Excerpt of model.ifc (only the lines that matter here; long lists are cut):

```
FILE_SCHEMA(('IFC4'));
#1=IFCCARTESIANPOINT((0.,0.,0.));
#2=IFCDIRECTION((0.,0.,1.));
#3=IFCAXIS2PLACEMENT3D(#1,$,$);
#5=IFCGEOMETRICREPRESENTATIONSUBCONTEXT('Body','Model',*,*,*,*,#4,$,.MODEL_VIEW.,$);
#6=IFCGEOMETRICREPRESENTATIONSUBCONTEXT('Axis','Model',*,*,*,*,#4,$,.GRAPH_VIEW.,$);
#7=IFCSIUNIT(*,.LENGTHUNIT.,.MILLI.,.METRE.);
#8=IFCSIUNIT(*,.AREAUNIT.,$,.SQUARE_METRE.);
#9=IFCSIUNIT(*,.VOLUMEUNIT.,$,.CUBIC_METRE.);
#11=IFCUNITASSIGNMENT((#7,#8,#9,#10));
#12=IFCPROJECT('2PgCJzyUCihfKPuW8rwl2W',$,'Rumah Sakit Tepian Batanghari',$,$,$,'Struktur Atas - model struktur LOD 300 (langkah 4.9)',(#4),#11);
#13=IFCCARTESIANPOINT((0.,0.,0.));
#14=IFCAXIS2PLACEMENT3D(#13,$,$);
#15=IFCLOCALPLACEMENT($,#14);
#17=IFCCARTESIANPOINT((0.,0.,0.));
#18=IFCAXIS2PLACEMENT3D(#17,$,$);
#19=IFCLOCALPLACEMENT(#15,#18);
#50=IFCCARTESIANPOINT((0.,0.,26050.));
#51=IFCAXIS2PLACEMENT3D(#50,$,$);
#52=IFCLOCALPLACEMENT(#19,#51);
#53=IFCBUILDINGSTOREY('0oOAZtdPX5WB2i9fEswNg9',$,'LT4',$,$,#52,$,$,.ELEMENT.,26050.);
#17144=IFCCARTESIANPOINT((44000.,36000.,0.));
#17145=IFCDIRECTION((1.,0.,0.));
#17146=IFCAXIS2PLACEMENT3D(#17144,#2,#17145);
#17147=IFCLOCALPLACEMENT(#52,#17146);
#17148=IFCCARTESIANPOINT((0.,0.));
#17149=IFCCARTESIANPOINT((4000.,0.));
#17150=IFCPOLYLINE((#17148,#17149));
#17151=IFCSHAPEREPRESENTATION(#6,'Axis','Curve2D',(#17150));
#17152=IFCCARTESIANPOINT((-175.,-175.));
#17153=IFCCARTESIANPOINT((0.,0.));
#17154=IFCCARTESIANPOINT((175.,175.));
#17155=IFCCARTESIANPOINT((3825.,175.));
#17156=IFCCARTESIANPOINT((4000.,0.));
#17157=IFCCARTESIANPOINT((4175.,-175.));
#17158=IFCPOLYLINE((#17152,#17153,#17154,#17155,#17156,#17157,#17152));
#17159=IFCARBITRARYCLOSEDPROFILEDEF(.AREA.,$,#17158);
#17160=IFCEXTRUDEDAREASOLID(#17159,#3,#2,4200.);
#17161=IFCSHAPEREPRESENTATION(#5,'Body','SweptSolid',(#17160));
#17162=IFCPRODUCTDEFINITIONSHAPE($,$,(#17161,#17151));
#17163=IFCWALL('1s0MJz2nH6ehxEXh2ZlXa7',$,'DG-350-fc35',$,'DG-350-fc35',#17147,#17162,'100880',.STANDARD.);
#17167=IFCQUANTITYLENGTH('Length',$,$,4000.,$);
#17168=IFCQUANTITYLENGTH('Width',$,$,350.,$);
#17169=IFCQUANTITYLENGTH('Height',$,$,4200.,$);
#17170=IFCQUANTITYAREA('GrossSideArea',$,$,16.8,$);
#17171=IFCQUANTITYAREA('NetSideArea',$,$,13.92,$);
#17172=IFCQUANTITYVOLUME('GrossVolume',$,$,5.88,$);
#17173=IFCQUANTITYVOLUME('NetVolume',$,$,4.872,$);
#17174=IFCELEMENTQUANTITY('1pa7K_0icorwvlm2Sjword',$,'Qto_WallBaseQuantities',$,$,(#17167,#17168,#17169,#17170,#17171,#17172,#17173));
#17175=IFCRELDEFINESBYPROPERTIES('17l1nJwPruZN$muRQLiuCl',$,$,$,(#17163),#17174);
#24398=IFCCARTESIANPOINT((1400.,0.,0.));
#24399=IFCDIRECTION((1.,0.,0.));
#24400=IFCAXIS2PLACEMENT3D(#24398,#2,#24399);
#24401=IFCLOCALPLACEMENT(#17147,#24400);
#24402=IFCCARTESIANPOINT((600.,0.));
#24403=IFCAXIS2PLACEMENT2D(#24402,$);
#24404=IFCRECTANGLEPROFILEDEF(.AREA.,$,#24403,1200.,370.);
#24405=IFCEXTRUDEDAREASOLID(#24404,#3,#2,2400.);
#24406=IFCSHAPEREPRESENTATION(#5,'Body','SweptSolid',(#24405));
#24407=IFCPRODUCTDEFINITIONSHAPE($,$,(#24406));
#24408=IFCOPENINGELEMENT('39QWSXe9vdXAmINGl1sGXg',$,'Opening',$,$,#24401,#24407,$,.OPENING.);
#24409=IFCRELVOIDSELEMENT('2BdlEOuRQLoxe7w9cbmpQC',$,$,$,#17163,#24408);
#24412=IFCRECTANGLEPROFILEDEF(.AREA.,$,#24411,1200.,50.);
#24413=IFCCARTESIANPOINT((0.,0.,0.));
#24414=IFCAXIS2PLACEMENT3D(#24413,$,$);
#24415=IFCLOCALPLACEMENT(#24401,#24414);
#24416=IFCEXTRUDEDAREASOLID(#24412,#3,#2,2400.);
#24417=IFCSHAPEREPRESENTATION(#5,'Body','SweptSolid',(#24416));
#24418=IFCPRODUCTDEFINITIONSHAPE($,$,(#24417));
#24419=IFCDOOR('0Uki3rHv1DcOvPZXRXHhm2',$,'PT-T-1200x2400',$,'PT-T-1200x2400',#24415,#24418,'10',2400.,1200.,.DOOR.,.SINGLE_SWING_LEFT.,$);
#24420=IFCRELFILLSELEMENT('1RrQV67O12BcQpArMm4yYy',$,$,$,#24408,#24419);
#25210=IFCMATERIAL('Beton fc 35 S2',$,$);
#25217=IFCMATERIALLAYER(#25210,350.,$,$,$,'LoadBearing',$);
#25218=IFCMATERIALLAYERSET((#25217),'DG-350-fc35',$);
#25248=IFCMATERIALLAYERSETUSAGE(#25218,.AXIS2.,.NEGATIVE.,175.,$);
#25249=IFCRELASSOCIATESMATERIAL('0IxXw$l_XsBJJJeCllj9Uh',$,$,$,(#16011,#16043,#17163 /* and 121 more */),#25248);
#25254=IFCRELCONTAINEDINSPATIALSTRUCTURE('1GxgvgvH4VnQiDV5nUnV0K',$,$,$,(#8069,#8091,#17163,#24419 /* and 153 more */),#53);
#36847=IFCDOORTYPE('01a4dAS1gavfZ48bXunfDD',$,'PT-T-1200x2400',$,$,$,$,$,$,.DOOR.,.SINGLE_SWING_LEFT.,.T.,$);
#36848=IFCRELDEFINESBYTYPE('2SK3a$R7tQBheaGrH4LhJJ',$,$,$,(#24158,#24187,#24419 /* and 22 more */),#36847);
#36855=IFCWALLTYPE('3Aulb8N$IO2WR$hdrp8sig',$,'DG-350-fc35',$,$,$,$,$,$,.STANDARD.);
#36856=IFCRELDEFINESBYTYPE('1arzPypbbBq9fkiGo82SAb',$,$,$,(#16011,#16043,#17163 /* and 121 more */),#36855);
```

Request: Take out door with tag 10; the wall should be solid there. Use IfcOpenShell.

```python
import ifcopenshell
import ifcopenshell.api.feature
import ifcopenshell.api.pset
import ifcopenshell.api.root
import ifcopenshell.geom
import ifcopenshell.util.element
import ifcopenshell.util.shape
import ifcopenshell.util.unit

model = ifcopenshell.open("model.ifc")
area_scale = ifcopenshell.util.unit.calculate_unit_scale(model, "AREAUNIT")
volume_scale = ifcopenshell.util.unit.calculate_unit_scale(model, "VOLUMEUNIT")
settings = ifcopenshell.geom.settings()


def volume(element):
    """Net volume in cubic metres, openings subtracted."""
    shape = ifcopenshell.geom.create_shape(settings, element)
    return ifcopenshell.util.shape.get_volume(shape.geometry)


door = model.by_guid("0Uki3rHv1DcOvPZXRXHhm2")
opening = door.FillsVoids[0].RelatingOpeningElement
wall = opening.VoidsElements[0].RelatingBuildingElement
before = volume(wall)

ifcopenshell.api.root.remove_product(model, product=door)
ifcopenshell.api.feature.remove_feature(model, feature=opening)

after = volume(wall)
thickness = 0.35  # wall thickness in metres

# Update the wall's stored quantities.
qto = model.by_id(ifcopenshell.util.element.get_pset(wall, "Qto_WallBaseQuantities", should_inherit=False)["id"])
ifcopenshell.api.pset.edit_qto(model, qto=qto, properties={
    "NetSideArea": after / thickness / area_scale,
    "NetVolume": after / volume_scale,
})

print(f"wall volume {before:.3f} -> {after:.3f} m3")

model.write("model_v2.ifc")
```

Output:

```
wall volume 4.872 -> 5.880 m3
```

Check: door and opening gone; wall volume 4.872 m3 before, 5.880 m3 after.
